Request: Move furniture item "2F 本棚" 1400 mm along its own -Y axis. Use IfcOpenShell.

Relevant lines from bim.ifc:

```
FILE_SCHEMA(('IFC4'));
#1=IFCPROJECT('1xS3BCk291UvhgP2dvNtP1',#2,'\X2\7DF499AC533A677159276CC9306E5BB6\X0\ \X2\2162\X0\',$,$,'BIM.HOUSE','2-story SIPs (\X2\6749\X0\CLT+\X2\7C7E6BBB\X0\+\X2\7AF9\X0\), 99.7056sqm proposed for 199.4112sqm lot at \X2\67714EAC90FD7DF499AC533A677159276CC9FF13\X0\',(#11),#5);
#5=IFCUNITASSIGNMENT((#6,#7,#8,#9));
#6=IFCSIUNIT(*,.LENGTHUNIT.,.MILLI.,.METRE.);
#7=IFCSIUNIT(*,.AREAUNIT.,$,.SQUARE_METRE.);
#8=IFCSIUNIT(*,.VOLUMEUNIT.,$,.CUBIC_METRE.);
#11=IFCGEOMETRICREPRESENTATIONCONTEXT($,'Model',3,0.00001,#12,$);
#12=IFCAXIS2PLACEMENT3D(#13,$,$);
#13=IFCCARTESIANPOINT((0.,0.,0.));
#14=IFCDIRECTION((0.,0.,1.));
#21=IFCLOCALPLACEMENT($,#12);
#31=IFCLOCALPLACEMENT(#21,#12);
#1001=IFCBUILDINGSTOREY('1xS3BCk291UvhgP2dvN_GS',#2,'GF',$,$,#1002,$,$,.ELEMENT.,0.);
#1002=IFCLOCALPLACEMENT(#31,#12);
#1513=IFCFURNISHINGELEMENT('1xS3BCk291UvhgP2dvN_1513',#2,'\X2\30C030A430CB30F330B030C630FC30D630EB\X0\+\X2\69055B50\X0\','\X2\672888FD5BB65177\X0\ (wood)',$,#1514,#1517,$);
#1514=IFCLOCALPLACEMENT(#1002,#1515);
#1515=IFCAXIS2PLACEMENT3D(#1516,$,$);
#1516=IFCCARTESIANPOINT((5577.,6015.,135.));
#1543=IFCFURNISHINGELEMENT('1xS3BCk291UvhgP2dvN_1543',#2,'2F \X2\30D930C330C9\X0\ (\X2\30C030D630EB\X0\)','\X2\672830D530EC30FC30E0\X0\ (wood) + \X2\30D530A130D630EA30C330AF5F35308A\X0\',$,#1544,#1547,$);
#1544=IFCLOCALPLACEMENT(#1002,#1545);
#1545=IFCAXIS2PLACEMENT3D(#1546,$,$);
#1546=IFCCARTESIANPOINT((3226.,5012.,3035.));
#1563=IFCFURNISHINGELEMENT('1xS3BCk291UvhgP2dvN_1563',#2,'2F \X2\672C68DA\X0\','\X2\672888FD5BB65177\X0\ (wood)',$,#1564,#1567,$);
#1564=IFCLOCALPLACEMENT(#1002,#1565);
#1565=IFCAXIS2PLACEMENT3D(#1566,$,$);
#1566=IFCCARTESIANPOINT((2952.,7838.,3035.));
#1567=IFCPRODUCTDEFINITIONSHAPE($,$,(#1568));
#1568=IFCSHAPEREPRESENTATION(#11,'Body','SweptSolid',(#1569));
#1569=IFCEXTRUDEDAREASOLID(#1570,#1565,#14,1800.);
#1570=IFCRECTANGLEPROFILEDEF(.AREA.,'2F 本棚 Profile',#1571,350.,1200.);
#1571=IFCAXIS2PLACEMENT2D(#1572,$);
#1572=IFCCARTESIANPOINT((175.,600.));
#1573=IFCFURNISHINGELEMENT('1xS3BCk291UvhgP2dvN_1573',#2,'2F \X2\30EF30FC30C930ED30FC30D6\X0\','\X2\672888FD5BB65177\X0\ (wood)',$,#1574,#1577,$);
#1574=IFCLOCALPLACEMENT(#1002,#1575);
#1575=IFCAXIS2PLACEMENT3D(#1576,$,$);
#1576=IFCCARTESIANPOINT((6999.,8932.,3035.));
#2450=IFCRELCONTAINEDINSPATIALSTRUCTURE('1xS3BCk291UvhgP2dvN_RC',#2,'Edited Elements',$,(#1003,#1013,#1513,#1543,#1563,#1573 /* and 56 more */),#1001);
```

```python
import ifcopenshell
import ifcopenshell.api.geometry
import ifcopenshell.util.placement
import ifcopenshell.util.unit

model = ifcopenshell.open("bim.ifc")
unit_scale = ifcopenshell.util.unit.calculate_unit_scale(model)

item = model.by_guid("1xS3BCk291UvhgP2dvN_1563")
matrix = ifcopenshell.util.placement.get_local_placement(item.ObjectPlacement)
matrix[:3, 3] -= matrix[:3, 1] * 1.4 / unit_scale
ifcopenshell.api.geometry.edit_object_placement(model, product=item, matrix=matrix, is_si=False)

print(ifcopenshell.util.placement.get_local_placement(item.ObjectPlacement).round(3) + 0.0)

model.write("bim_v2.ifc")
```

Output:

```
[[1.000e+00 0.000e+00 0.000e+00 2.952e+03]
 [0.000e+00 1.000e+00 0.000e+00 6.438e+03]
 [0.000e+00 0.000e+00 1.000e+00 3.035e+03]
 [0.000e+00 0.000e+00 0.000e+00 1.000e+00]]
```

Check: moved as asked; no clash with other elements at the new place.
